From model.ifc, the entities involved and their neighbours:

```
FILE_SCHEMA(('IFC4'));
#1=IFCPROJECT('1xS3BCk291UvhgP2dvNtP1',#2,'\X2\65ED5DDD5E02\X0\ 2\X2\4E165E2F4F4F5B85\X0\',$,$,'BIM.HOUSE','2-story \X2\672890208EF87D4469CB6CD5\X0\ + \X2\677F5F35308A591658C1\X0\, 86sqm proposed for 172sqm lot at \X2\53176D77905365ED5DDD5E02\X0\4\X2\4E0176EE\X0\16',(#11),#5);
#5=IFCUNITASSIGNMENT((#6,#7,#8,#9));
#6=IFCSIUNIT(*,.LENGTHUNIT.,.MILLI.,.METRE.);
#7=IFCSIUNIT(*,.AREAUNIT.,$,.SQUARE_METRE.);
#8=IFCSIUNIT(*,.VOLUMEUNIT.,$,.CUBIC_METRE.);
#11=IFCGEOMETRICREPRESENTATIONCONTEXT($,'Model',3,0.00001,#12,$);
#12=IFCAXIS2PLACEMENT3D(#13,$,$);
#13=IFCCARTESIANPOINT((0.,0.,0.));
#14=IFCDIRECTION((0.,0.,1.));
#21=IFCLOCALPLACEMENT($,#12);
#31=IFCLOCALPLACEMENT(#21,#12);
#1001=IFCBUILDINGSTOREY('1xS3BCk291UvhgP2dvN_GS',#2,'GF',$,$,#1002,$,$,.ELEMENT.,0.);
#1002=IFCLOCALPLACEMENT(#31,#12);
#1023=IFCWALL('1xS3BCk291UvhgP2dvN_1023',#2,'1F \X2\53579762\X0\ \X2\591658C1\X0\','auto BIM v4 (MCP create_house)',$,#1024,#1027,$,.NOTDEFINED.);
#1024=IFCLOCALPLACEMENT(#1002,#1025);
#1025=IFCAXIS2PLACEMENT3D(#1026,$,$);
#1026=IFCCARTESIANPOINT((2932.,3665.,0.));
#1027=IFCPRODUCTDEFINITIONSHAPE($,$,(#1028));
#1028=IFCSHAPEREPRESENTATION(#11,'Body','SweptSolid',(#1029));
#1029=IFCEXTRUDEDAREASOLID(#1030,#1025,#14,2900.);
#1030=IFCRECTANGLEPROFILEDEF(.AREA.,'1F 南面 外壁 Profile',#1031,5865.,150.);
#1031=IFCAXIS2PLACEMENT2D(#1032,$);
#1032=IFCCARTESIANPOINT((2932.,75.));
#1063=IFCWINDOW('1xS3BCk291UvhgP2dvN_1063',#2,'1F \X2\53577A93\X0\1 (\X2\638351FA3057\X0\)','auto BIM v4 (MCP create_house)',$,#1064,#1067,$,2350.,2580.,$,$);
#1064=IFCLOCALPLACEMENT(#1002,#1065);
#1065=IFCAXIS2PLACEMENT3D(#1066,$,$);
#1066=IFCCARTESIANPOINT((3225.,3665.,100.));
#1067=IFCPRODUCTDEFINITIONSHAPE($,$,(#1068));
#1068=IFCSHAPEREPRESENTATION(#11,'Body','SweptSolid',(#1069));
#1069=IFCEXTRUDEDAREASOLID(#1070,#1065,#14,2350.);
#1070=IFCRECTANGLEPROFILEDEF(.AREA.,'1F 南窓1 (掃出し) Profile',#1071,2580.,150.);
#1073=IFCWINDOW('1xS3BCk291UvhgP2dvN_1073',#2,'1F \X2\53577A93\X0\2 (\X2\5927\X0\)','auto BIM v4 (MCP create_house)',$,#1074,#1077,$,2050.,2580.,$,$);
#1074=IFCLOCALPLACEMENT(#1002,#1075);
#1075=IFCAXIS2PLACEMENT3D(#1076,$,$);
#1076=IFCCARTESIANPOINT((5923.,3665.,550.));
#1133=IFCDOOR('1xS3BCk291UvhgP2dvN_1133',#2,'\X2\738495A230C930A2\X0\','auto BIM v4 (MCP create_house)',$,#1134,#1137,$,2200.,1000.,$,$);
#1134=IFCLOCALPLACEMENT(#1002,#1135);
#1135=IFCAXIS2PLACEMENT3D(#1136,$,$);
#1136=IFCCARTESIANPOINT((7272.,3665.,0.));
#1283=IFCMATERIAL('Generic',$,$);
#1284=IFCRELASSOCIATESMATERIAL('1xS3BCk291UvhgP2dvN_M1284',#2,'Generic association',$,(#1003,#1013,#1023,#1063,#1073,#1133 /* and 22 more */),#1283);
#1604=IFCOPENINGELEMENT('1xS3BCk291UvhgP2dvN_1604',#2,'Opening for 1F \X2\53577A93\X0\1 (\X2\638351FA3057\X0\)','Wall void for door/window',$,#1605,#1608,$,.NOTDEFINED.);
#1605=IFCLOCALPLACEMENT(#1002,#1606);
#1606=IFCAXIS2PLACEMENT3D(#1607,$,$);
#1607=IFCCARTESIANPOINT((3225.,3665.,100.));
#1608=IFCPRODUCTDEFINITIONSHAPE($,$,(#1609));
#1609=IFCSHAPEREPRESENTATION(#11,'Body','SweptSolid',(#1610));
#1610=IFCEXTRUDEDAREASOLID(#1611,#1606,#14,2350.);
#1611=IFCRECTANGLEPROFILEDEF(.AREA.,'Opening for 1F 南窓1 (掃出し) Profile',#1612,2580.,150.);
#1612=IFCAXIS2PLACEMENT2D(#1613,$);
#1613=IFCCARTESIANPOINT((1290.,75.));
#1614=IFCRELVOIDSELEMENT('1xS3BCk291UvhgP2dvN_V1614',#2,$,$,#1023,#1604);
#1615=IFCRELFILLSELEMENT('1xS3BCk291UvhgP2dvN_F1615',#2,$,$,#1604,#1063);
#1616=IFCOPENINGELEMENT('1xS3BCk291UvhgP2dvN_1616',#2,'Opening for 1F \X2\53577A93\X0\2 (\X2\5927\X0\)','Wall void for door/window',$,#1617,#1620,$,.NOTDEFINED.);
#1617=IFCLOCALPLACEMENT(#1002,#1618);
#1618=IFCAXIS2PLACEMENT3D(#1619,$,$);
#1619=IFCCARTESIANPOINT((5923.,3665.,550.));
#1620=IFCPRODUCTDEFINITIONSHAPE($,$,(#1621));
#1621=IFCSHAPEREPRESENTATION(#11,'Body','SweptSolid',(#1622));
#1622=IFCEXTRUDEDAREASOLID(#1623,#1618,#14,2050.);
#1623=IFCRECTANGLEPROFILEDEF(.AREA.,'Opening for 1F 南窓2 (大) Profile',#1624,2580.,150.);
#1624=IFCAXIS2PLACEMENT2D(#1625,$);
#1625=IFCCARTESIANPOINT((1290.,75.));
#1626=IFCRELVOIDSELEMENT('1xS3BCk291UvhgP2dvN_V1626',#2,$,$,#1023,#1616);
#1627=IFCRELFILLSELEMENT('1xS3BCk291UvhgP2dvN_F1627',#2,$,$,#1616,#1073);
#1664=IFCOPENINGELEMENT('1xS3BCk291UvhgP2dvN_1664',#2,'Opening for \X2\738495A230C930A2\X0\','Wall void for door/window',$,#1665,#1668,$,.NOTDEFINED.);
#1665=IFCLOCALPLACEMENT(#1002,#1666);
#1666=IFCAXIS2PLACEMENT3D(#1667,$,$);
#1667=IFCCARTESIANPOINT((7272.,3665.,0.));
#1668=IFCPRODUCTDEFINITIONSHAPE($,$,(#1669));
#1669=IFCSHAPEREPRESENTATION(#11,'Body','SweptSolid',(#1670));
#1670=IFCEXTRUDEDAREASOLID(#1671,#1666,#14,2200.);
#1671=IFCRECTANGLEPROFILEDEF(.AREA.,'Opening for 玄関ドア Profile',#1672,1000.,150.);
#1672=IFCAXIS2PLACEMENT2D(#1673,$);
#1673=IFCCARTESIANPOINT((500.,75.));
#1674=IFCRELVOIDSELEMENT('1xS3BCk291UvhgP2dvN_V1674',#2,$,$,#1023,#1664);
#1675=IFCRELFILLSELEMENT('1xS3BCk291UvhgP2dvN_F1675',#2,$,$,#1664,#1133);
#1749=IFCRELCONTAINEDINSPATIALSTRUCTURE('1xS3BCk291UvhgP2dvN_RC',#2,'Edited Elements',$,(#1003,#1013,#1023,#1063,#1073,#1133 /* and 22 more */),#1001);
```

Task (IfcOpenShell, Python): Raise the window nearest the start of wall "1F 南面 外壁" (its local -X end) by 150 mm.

```python
import numpy as np
import ifcopenshell
import ifcopenshell.api.geometry
import ifcopenshell.util.placement
import ifcopenshell.util.unit

model = ifcopenshell.open("model.ifc")
unit_scale = ifcopenshell.util.unit.calculate_unit_scale(model)

window = model.by_guid("1xS3BCk291UvhgP2dvN_1063")
opening = window.FillsVoids[0].RelatingOpeningElement
dz = 150.0

shift = np.array([0.0, 0.0, dz])
# The window is not placed relative to its opening, so move both.
for product in (opening, window):
    matrix = ifcopenshell.util.placement.get_local_placement(product.ObjectPlacement)
    matrix[:3, 3] += shift
    ifcopenshell.api.geometry.edit_object_placement(model, product=product, matrix=matrix, is_si=False)

print(f"moved by {dz * unit_scale:+.3f} m")

model.write("model_edited.ifc")
```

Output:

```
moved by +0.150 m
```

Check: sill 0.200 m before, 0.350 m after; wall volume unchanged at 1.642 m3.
